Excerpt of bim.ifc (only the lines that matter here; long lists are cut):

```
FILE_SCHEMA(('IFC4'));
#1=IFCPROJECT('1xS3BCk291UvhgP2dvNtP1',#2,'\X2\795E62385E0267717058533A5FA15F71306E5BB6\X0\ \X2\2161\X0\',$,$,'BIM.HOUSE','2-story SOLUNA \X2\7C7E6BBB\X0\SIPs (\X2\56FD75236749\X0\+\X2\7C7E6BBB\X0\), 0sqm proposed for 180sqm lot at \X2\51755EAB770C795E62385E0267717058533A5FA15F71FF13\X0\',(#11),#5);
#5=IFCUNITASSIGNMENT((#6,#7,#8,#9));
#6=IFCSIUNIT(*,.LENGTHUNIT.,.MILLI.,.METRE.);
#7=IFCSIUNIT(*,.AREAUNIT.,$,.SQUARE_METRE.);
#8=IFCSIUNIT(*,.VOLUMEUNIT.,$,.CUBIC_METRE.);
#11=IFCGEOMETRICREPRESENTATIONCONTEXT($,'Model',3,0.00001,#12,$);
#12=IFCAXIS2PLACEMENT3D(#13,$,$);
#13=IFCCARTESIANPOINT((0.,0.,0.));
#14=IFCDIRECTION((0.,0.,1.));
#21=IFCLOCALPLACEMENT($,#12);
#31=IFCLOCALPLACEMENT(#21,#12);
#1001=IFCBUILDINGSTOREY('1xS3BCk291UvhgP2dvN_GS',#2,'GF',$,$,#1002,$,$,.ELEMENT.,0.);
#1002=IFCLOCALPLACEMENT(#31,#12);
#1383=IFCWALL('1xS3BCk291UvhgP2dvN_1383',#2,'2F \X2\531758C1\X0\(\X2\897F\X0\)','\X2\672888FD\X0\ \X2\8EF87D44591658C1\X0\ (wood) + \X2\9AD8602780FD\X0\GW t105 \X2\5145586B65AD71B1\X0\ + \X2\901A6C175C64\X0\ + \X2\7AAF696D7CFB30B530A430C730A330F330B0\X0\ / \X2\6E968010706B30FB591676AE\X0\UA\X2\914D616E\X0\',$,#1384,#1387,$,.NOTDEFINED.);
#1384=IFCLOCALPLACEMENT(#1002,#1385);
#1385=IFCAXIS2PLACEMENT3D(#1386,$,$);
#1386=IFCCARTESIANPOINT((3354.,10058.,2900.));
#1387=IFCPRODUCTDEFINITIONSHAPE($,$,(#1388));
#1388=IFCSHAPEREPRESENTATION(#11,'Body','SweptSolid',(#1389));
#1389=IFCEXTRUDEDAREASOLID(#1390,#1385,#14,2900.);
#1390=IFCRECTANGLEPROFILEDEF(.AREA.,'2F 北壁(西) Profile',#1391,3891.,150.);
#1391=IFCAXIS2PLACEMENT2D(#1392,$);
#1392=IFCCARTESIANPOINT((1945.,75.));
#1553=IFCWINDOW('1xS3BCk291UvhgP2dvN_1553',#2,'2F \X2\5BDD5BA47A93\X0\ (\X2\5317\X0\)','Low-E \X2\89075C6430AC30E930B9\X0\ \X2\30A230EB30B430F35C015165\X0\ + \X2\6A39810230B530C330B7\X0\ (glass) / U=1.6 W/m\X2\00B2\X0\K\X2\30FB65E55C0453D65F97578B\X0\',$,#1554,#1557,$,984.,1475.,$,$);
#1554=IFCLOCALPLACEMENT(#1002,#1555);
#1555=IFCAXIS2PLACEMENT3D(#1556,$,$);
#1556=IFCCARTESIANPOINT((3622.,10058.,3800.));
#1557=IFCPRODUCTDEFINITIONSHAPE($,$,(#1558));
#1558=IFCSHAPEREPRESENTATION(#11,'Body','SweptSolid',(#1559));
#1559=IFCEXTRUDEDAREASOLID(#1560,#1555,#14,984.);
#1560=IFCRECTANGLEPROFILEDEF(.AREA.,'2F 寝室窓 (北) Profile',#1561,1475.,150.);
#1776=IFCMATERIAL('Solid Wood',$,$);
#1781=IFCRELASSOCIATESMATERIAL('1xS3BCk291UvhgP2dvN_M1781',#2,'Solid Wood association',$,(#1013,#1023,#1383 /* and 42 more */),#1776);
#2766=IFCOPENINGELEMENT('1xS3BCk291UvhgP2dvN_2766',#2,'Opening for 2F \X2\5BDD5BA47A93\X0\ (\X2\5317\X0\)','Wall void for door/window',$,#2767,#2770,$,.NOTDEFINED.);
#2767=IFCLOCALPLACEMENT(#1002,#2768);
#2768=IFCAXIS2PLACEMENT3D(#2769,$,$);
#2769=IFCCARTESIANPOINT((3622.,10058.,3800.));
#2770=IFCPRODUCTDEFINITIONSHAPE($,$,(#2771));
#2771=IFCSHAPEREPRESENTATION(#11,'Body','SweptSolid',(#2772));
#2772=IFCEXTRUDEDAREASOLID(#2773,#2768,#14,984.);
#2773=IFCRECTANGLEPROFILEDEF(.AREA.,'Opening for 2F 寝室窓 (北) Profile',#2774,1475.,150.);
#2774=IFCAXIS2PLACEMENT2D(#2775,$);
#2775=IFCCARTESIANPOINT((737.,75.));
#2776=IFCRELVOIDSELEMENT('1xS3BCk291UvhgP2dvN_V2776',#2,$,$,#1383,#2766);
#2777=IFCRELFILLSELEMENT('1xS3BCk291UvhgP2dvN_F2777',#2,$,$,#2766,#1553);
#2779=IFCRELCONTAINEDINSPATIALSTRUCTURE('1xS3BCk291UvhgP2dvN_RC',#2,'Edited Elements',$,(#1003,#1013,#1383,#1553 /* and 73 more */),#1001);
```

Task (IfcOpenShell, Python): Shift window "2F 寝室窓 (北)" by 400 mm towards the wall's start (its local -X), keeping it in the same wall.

```python
import ifcopenshell
import ifcopenshell.api.geometry
import ifcopenshell.util.placement

model = ifcopenshell.open("bim.ifc")

window = model.by_guid("1xS3BCk291UvhgP2dvN_1553")
opening = window.FillsVoids[0].RelatingOpeningElement
wall = opening.VoidsElements[0].RelatingBuildingElement

wall_matrix = ifcopenshell.util.placement.get_local_placement(wall.ObjectPlacement)
shift = wall_matrix[:3, 0] * -400.0
before = ifcopenshell.util.placement.get_local_placement(window.ObjectPlacement)[:3, 3].copy()

# The window is not placed relative to its opening, so move both.
for product in (opening, window):
    matrix = ifcopenshell.util.placement.get_local_placement(product.ObjectPlacement)
    matrix[:3, 3] += shift
    ifcopenshell.api.geometry.edit_object_placement(model, product=product, matrix=matrix, is_si=False)

after = ifcopenshell.util.placement.get_local_placement(window.ObjectPlacement)[:3, 3]
print("window moved by", (after - before).round(3) + 0.0)

model.write("bim_rev.ifc")
```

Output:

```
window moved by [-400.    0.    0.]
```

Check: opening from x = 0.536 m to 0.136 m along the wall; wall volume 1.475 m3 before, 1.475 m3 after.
